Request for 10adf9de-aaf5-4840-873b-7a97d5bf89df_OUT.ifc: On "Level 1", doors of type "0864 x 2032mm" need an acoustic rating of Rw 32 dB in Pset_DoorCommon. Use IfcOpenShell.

First a look at what the model holds.

```python
import ifcopenshell
import ifcopenshell.util.element

model = ifcopenshell.open("10adf9de-aaf5-4840-873b-7a97d5bf89df_OUT.ifc")
print(model.schema)
storey = next(s for s in model.by_type("IfcBuildingStorey") if s.Name == "Level 1")
doors = [e for e in ifcopenshell.util.element.get_decomposition(storey) if e.is_a("IfcDoor")]
seen = {}
for e in doors:
    element_type = ifcopenshell.util.element.get_type(e)
    key = (element_type.Name if element_type != e and element_type else None, ifcopenshell.util.element.get_pset(e, "Pset_DoorCommon", "AcousticRating"))
    seen[key] = seen.get(key, 0) + 1
for (name, value), count in sorted(seen.items(), key=str):
    print(count, "x", name, "|", value)
```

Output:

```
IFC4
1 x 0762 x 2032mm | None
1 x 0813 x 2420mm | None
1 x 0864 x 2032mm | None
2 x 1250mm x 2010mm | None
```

```python
import ifcopenshell
import ifcopenshell.api.pset
import ifcopenshell.util.element

model = ifcopenshell.open("10adf9de-aaf5-4840-873b-7a97d5bf89df_OUT.ifc")

storey = next(s for s in model.by_type("IfcBuildingStorey") if s.Name == "Level 1")
doors = [e for e in ifcopenshell.util.element.get_decomposition(storey) if e.is_a("IfcDoor")]

count = 0
for e in doors:
    element_type = ifcopenshell.util.element.get_type(e)
    if element_type in (None, e) or element_type.Name != "0864 x 2032mm":
        continue
    # add_pset returns the element's existing set when there is one.
    pset = ifcopenshell.api.pset.add_pset(model, product=e, name="Pset_DoorCommon")
    ifcopenshell.api.pset.edit_pset(model, pset=pset, properties={"AcousticRating": "Rw 32 dB"})
    count += 1

print(count, "doors updated")

model.write("10adf9de-aaf5-4840-873b-7a97d5bf89df_OUT-out.ifc")
```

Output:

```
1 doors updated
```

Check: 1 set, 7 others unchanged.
